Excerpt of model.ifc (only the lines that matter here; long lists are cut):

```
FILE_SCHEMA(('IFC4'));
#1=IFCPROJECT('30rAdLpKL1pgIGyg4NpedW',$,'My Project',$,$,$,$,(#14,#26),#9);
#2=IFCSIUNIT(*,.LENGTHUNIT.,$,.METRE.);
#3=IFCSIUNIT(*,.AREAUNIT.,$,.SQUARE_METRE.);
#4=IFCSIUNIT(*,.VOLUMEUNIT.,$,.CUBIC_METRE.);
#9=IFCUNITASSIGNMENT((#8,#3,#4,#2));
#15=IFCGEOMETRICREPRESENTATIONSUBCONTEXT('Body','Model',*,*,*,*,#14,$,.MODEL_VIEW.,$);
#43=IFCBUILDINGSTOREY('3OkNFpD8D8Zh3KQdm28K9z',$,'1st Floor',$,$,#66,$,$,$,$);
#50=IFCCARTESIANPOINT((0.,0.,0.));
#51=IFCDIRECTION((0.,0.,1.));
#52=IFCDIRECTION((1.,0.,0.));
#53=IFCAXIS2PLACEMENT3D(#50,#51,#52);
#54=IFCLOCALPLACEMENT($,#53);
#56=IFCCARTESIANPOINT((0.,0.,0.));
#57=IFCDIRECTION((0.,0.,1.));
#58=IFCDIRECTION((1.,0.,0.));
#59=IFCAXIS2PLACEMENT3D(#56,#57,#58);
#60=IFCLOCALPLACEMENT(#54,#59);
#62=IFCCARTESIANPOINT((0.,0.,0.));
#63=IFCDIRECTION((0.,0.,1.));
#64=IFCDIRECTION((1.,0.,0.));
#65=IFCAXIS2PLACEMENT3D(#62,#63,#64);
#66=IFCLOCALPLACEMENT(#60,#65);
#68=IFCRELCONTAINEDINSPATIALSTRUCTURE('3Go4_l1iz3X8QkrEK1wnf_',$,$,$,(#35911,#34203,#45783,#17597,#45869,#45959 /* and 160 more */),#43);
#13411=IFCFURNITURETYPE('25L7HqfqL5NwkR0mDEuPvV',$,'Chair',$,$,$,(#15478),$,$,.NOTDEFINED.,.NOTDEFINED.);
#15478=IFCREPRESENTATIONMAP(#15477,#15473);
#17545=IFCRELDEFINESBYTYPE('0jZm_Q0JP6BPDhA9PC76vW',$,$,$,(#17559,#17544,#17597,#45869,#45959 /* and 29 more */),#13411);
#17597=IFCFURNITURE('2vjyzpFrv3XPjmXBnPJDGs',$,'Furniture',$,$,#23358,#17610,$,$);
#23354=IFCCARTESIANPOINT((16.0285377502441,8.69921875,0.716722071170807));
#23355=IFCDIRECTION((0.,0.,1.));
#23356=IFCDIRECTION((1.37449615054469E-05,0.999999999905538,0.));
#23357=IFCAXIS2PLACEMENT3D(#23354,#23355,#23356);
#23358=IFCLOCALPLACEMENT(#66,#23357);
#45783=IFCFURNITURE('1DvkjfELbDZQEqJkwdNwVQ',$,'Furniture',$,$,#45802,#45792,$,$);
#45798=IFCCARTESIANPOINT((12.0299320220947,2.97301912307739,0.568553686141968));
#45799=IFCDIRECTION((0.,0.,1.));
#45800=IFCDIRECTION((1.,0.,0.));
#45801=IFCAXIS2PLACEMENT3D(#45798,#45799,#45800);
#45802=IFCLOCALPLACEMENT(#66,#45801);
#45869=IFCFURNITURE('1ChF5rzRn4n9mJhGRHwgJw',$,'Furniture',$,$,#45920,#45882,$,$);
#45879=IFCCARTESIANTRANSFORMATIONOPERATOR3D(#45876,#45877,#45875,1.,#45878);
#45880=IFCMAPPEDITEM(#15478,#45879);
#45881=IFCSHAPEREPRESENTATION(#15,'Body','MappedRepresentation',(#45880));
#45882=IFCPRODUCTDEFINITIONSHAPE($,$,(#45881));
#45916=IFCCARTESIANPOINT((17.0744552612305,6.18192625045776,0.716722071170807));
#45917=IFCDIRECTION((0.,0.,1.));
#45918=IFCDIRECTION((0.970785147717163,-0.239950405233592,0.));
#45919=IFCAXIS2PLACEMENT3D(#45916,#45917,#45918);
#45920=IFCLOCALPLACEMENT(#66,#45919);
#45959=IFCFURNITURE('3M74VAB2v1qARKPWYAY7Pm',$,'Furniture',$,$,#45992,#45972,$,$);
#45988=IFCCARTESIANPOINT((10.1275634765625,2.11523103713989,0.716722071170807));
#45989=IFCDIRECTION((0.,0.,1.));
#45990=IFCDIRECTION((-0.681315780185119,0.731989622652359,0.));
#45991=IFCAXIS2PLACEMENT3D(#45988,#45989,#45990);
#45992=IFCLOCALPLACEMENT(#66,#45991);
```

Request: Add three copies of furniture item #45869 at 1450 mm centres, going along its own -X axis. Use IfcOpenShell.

```python
import ifcopenshell
import ifcopenshell.api.geometry
import ifcopenshell.api.root
import ifcopenshell.util.element
import ifcopenshell.util.placement

model = ifcopenshell.open("model.ifc")

source = model.by_guid("1ChF5rzRn4n9mJhGRHwgJw")
base = ifcopenshell.util.placement.get_local_placement(source.ObjectPlacement)
step = -base[:3, 0] * 1.45

for i in range(1, 4):
    copy = ifcopenshell.api.root.copy_class(model, product=source)
    copy.Representation = ifcopenshell.util.element.copy_deep(
        model, source.Representation, exclude=["IfcGeometricRepresentationContext", "IfcRepresentationMap"]
    )
    matrix = base.copy()
    matrix[:3, 3] += i * step
    print("added at", matrix[:3, 3].round(3) + 0.0)
    ifcopenshell.api.geometry.edit_object_placement(model, product=copy, matrix=matrix, is_si=False)

model.write("model_rev.ifc")
```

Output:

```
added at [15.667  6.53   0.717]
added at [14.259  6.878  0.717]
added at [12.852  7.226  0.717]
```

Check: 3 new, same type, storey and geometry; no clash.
